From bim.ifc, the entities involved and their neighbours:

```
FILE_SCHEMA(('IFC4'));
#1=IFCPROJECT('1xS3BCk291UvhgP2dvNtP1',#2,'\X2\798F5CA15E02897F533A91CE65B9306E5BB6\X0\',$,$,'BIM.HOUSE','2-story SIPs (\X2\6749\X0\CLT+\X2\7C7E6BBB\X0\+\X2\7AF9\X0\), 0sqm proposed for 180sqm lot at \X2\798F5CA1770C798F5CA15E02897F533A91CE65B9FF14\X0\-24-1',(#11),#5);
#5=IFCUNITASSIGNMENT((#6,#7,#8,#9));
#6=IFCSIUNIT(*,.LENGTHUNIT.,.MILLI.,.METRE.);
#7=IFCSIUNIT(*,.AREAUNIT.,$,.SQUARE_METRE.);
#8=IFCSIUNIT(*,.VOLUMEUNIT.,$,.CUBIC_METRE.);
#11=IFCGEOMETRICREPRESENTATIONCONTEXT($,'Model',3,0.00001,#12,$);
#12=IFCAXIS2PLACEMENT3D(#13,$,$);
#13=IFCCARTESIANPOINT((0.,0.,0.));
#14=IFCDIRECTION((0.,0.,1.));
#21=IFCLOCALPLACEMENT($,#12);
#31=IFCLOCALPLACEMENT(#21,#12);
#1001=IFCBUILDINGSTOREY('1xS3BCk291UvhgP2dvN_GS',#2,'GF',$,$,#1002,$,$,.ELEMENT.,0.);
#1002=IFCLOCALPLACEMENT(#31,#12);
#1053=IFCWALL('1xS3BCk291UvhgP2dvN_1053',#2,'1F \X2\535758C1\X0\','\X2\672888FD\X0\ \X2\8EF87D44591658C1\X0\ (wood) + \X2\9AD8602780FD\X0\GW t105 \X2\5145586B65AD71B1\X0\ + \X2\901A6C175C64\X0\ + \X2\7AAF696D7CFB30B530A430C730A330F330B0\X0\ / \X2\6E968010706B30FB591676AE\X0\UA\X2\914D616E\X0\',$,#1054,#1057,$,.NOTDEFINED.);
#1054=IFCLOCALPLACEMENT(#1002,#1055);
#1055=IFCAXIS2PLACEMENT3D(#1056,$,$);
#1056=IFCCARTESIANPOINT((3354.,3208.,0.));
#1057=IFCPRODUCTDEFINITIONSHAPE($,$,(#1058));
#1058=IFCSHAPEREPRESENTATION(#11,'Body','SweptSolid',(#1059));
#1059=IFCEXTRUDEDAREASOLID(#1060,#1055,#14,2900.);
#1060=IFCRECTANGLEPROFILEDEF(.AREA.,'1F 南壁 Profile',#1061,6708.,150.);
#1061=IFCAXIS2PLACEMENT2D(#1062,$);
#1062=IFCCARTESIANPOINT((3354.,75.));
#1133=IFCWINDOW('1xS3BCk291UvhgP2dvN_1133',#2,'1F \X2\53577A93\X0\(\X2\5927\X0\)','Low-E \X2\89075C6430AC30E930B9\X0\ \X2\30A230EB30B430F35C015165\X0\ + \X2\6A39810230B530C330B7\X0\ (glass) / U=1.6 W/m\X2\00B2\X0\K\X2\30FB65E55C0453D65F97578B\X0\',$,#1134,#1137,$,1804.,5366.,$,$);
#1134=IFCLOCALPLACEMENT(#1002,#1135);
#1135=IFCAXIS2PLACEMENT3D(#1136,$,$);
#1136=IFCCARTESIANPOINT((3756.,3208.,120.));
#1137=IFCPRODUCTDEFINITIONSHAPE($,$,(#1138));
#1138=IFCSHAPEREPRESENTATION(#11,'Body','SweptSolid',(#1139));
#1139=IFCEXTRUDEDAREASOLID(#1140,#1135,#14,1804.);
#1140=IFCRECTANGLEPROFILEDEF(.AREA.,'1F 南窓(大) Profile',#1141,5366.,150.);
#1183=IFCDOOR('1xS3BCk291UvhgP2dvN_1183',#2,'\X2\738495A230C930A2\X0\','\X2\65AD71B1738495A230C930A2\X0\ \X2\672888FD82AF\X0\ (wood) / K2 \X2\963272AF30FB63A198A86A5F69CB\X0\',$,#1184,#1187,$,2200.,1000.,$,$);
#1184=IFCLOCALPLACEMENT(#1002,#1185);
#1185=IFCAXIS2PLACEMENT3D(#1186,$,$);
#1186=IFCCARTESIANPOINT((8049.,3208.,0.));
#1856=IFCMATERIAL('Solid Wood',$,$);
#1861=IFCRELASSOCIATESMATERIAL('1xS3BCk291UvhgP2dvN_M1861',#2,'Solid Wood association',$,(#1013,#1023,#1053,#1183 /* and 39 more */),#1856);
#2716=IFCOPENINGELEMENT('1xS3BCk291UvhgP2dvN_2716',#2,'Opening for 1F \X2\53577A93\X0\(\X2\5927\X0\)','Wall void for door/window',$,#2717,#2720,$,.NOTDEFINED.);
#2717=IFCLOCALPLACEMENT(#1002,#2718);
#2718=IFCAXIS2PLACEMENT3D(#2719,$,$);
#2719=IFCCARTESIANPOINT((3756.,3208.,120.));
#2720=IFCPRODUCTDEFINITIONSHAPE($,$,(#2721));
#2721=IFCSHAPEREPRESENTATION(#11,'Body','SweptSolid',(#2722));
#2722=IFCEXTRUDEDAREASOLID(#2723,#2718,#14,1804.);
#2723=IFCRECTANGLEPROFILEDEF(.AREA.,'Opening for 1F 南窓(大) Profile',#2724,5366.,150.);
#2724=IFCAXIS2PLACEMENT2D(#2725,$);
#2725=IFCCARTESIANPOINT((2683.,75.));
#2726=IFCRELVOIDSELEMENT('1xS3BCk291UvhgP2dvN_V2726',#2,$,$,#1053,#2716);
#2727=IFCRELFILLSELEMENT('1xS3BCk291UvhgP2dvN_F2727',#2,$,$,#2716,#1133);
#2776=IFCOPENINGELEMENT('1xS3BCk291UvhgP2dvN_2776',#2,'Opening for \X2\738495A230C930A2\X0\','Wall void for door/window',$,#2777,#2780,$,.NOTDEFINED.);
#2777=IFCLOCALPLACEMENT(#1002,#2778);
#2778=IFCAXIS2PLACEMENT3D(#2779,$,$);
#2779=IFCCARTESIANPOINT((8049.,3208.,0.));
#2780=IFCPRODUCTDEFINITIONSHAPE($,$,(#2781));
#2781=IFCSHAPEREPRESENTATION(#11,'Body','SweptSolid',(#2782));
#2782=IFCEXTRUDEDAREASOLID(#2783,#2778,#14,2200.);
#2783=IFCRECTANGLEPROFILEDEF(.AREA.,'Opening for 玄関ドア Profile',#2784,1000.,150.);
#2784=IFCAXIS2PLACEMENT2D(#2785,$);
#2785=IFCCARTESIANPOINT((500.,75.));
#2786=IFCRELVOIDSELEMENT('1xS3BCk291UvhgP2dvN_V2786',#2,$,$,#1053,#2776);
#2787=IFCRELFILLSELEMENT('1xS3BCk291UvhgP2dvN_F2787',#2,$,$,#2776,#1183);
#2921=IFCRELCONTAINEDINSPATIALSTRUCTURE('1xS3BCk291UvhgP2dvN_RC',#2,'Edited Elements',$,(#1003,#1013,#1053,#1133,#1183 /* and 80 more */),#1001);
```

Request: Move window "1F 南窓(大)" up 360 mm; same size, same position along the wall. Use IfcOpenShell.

```python
import numpy as np
import ifcopenshell
import ifcopenshell.api.geometry
import ifcopenshell.util.placement
import ifcopenshell.util.unit

model = ifcopenshell.open("bim.ifc")
unit_scale = ifcopenshell.util.unit.calculate_unit_scale(model)

window = model.by_id(1133)
opening = window.FillsVoids[0].RelatingOpeningElement
dz = 360.0

shift = np.array([0.0, 0.0, dz])
# The window is not placed relative to its opening, so move both.
for product in (opening, window):
    matrix = ifcopenshell.util.placement.get_local_placement(product.ObjectPlacement)
    matrix[:3, 3] += shift
    ifcopenshell.api.geometry.edit_object_placement(model, product=product, matrix=matrix, is_si=False)

print(f"moved by {dz * unit_scale:+.3f} m")

model.write("bim_v2.ifc")
```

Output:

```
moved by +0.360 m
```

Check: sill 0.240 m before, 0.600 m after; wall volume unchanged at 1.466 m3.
